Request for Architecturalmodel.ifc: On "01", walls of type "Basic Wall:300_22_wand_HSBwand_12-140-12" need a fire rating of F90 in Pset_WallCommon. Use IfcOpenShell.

First a look at what the model holds.

```python
import ifcopenshell
import ifcopenshell.util.element

model = ifcopenshell.open("Architecturalmodel.ifc")
print(model.schema)
storey = next(s for s in model.by_type("IfcBuildingStorey") if s.Name == "01")
walls = [e for e in ifcopenshell.util.element.get_decomposition(storey) if e.is_a("IfcWall")]
seen = {}
for e in walls:
    element_type = ifcopenshell.util.element.get_type(e)
    key = (element_type.Name if element_type != e and element_type else None, ifcopenshell.util.element.get_pset(e, "Pset_WallCommon", "FireRating"))
    seen[key] = seen.get(key, 0) + 1
for (name, value), count in sorted(seen.items(), key=str):
    print(count, "x", name, "|", value)
```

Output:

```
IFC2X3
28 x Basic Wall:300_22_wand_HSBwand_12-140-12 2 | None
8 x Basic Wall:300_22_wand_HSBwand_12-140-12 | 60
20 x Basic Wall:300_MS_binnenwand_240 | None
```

```python
import ifcopenshell
import ifcopenshell.api.pset
import ifcopenshell.util.element

model = ifcopenshell.open("Architecturalmodel.ifc")

storey = next(s for s in model.by_type("IfcBuildingStorey") if s.Name == "01")
walls = [e for e in ifcopenshell.util.element.get_decomposition(storey) if e.is_a("IfcWall")]

count = 0
for e in walls:
    element_type = ifcopenshell.util.element.get_type(e)
    if element_type in (None, e) or element_type.Name != "Basic Wall:300_22_wand_HSBwand_12-140-12":
        continue
    # add_pset returns the element's existing set when there is one.
    pset = ifcopenshell.api.pset.add_pset(model, product=e, name="Pset_WallCommon")
    ifcopenshell.api.pset.edit_pset(model, pset=pset, properties={"FireRating": "F90"})
    count += 1

print(count, "walls updated")

model.write("Architecturalmodel_v2.ifc")
```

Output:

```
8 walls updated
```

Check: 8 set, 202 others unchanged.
